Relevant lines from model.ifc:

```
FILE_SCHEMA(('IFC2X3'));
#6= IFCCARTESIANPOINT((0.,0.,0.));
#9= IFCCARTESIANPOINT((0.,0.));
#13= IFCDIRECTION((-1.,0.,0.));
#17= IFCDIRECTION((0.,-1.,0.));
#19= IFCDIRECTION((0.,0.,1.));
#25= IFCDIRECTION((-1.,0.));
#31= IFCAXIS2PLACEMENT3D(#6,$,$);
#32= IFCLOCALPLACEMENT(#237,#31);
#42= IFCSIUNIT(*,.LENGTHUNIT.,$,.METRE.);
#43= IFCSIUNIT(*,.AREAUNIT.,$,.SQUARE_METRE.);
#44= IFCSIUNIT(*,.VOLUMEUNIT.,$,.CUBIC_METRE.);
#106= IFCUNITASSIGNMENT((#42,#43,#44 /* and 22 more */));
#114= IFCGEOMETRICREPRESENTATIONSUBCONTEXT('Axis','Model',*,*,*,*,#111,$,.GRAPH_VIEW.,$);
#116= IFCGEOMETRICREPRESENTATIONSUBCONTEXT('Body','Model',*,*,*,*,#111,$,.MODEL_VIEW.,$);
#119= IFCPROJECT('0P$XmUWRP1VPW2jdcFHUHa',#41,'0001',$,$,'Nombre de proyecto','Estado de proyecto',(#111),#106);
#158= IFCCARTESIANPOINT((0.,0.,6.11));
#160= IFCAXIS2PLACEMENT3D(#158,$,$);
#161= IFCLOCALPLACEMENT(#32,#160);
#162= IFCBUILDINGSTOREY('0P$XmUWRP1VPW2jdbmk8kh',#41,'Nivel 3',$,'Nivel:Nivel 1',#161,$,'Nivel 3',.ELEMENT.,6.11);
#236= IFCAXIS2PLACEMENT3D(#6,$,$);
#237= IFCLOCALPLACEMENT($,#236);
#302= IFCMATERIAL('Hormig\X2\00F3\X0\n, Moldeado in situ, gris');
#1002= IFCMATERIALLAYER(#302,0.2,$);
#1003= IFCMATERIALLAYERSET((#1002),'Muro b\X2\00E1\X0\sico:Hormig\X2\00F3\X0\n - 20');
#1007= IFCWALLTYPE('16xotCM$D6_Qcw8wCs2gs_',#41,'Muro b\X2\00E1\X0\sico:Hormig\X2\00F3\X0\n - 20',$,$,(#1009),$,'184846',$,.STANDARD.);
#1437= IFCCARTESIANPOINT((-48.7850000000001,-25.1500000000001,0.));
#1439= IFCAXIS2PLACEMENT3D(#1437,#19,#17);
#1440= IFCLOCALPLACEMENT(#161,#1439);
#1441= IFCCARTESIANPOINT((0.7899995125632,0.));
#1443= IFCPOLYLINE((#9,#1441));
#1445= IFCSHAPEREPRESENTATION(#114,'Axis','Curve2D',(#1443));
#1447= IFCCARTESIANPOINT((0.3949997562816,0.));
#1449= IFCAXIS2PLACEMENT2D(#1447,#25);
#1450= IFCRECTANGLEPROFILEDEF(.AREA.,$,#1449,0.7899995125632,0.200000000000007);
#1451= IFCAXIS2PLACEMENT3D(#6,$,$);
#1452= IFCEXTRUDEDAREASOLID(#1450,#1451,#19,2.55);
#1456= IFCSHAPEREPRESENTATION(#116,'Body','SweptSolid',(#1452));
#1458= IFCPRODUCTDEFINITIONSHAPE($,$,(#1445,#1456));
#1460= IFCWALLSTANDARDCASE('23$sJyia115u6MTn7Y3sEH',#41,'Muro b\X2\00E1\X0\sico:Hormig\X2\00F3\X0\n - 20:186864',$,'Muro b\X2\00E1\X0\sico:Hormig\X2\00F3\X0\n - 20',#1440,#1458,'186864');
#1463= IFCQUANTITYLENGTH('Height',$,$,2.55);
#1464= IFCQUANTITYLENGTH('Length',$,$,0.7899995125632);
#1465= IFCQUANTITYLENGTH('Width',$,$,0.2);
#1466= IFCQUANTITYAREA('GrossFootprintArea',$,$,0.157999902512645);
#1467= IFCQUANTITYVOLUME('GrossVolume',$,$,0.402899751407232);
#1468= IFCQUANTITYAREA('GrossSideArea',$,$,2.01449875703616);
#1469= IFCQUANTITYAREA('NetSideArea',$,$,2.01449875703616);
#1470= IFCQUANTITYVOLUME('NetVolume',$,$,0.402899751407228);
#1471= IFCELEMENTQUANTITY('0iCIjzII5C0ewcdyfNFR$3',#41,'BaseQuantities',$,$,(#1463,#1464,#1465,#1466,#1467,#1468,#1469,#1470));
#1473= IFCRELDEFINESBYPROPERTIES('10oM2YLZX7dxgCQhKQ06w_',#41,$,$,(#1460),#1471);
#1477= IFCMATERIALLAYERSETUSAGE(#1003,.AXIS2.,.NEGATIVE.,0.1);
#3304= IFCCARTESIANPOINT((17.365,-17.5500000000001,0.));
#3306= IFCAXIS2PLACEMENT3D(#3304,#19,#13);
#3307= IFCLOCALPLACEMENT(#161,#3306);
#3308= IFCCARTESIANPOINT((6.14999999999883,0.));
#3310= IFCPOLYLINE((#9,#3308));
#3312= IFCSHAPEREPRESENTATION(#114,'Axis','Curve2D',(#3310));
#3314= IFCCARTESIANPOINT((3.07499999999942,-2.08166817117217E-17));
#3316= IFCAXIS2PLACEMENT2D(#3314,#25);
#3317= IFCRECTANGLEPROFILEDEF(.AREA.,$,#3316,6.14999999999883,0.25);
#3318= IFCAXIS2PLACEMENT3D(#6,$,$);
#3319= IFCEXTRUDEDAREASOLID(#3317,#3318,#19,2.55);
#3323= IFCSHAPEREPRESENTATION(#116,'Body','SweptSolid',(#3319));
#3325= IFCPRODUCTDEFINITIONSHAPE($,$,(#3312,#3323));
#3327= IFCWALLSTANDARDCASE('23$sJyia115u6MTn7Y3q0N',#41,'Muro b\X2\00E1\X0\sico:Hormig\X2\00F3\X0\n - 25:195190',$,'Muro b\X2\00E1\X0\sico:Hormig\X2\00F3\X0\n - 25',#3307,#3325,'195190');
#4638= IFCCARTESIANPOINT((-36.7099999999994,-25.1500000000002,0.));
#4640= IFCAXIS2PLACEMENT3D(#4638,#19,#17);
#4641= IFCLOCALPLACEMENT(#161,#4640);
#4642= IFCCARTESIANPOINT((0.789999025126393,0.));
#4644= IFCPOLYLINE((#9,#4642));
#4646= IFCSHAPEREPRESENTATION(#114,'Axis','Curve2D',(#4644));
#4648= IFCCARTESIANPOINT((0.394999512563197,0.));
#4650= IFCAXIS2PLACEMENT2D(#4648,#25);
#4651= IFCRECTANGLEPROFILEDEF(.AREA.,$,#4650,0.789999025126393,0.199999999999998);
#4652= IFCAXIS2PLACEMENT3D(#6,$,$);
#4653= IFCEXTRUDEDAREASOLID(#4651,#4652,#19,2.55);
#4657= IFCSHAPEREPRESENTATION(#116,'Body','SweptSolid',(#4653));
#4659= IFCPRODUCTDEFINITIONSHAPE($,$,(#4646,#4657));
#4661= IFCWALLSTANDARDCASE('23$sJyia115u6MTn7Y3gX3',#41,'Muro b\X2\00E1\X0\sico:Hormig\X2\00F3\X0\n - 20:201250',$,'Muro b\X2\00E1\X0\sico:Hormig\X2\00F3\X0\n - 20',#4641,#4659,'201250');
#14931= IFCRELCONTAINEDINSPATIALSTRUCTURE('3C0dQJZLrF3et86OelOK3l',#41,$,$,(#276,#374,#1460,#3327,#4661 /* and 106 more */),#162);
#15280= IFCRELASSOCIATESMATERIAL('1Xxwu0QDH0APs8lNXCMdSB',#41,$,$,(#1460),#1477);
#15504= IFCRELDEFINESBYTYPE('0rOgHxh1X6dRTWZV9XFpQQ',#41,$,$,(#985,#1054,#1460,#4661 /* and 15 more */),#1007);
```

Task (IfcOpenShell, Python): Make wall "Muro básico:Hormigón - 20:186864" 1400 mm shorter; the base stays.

```python
import ifcopenshell
import ifcopenshell.api.pset
import ifcopenshell.geom
import ifcopenshell.util.element
import ifcopenshell.util.representation
import ifcopenshell.util.shape
import ifcopenshell.util.unit

model = ifcopenshell.open("model.ifc")
unit_scale = ifcopenshell.util.unit.calculate_unit_scale(model)
area_scale = ifcopenshell.util.unit.calculate_unit_scale(model, "AREAUNIT")
volume_scale = ifcopenshell.util.unit.calculate_unit_scale(model, "VOLUMEUNIT")
settings = ifcopenshell.geom.settings()


def volume(element):
    """Net volume in cubic metres, openings subtracted."""
    shape = ifcopenshell.geom.create_shape(settings, element)
    return ifcopenshell.util.shape.get_volume(shape.geometry)


wall = model.by_id(1460)
before = volume(wall)

body = ifcopenshell.util.representation.get_representation(wall, "Model", "Body")
solid = body.Items[0]
old_height = solid.Depth
solid.Depth -= 1.4 / unit_scale
after = volume(wall)
thickness = 0.2  # wall thickness in metres

# Update the stored height, areas and volumes.
qto = model.by_id(ifcopenshell.util.element.get_pset(wall, "BaseQuantities", should_inherit=False)["id"])
ifcopenshell.api.pset.edit_qto(model, qto=qto, properties={
    "Height": solid.Depth,
    "GrossVolume": ifcopenshell.util.element.get_pset(wall, "BaseQuantities", "GrossVolume") * solid.Depth / old_height,
    "GrossSideArea": ifcopenshell.util.element.get_pset(wall, "BaseQuantities", "GrossSideArea") * solid.Depth / old_height,
    "NetSideArea": after / thickness / area_scale,
    "NetVolume": after / volume_scale,
})

print(f"height {old_height:g} -> {solid.Depth:g}, volume {before:.3f} -> {after:.3f} m3")

model.write("model_updated.ifc")
```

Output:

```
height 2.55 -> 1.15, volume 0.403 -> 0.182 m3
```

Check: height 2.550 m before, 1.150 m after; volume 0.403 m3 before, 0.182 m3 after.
